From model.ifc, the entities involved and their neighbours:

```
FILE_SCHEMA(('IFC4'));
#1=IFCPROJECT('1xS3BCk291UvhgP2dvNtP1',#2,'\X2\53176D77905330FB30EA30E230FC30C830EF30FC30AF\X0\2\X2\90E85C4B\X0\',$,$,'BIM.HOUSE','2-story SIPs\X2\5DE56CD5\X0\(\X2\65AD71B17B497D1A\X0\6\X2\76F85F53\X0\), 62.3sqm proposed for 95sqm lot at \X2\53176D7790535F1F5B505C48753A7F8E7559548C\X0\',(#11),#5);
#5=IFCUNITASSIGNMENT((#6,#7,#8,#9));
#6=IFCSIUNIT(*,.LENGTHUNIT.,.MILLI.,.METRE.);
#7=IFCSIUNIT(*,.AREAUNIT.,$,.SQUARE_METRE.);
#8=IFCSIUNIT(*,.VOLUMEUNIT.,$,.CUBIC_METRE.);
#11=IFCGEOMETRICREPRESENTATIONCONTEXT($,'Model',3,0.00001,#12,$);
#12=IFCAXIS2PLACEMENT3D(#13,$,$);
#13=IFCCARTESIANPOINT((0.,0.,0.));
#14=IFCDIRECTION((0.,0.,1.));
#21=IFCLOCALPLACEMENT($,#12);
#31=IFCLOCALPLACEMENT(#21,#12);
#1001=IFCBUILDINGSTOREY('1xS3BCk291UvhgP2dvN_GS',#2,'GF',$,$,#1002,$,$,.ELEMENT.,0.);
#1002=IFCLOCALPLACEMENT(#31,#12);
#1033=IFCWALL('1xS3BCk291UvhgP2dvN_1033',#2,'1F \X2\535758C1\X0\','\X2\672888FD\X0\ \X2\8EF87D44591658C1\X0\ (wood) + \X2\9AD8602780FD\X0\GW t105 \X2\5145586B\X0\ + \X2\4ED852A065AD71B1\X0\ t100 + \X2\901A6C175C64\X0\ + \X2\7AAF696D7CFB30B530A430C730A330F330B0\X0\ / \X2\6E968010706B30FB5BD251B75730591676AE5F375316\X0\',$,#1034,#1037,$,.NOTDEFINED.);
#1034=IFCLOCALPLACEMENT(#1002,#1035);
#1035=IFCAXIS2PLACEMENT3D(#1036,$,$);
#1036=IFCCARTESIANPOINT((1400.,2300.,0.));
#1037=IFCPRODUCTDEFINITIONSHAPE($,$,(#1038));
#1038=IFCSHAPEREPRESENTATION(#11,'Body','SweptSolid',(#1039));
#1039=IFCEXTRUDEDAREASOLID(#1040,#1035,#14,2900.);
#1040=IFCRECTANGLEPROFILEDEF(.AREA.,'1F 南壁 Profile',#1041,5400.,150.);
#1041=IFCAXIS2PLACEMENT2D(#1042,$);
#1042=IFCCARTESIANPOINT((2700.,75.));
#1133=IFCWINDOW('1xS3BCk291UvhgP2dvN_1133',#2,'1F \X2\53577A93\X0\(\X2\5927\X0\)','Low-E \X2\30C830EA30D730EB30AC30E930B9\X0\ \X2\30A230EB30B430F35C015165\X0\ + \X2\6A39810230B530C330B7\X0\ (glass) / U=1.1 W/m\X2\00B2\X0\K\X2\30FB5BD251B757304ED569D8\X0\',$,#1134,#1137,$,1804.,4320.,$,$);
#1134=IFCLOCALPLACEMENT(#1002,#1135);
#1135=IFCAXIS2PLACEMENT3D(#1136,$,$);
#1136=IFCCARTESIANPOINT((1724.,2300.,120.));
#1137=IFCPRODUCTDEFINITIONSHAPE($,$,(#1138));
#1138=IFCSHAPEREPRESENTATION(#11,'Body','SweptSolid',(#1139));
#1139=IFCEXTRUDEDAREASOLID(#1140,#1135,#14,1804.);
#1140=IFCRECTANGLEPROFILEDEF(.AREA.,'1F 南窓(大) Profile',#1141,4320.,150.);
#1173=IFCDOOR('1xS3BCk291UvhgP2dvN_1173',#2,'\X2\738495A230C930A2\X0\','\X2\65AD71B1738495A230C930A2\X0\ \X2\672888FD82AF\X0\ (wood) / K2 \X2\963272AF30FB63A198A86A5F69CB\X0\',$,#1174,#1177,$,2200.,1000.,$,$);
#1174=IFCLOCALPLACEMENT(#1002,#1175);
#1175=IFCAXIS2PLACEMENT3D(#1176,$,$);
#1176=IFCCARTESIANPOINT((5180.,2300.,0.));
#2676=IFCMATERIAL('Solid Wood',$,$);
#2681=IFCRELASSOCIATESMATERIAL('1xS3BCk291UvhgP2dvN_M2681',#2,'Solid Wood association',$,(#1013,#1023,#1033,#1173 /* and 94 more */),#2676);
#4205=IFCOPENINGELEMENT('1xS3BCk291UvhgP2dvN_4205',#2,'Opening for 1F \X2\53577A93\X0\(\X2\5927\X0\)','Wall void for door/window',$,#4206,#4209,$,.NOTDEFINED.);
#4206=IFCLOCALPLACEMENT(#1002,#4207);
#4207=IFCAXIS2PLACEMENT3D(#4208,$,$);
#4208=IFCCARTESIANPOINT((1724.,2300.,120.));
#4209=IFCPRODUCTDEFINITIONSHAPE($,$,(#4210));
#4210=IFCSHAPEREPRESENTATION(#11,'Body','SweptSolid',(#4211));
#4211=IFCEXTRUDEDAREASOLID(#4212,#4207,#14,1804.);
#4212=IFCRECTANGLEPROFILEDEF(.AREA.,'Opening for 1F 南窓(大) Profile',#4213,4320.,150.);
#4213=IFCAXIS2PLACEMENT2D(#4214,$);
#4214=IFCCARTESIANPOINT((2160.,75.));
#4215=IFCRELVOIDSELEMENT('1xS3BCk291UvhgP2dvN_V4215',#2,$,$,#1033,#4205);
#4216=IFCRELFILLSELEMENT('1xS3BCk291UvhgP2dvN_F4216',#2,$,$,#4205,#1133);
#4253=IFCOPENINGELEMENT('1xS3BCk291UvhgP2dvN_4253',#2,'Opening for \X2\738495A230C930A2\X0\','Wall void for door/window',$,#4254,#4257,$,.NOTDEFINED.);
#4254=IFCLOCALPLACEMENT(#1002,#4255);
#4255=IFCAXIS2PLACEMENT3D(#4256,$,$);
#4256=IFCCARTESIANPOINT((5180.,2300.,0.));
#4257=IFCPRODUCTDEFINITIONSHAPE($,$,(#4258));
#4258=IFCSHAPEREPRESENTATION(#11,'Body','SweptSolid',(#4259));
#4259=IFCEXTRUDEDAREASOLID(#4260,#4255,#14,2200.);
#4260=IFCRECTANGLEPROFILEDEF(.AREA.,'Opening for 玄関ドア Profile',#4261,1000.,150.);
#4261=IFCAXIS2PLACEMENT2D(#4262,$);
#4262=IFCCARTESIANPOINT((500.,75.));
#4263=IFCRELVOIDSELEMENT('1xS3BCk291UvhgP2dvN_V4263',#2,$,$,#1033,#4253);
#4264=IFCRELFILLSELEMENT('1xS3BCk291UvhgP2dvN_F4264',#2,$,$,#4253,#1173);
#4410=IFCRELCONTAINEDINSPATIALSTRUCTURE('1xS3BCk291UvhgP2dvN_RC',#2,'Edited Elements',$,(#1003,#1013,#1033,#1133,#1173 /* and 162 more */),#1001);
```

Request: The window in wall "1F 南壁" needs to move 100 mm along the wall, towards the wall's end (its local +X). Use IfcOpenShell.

```python
import ifcopenshell
import ifcopenshell.api.geometry
import ifcopenshell.util.placement

model = ifcopenshell.open("model.ifc")

window = model.by_guid("1xS3BCk291UvhgP2dvN_1133")
opening = window.FillsVoids[0].RelatingOpeningElement
wall = opening.VoidsElements[0].RelatingBuildingElement

wall_matrix = ifcopenshell.util.placement.get_local_placement(wall.ObjectPlacement)
shift = wall_matrix[:3, 0] * 100.0
before = ifcopenshell.util.placement.get_local_placement(window.ObjectPlacement)[:3, 3].copy()

# The window is not placed relative to its opening, so move both.
for product in (opening, window):
    matrix = ifcopenshell.util.placement.get_local_placement(product.ObjectPlacement)
    matrix[:3, 3] += shift
    ifcopenshell.api.geometry.edit_object_placement(model, product=product, matrix=matrix, is_si=False)

after = ifcopenshell.util.placement.get_local_placement(window.ObjectPlacement)[:3, 3]
print("window moved by", (after - before).round(3) + 0.0)

model.write("model_edited.ifc")
```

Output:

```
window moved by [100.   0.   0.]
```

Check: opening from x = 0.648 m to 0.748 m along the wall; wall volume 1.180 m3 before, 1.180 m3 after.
